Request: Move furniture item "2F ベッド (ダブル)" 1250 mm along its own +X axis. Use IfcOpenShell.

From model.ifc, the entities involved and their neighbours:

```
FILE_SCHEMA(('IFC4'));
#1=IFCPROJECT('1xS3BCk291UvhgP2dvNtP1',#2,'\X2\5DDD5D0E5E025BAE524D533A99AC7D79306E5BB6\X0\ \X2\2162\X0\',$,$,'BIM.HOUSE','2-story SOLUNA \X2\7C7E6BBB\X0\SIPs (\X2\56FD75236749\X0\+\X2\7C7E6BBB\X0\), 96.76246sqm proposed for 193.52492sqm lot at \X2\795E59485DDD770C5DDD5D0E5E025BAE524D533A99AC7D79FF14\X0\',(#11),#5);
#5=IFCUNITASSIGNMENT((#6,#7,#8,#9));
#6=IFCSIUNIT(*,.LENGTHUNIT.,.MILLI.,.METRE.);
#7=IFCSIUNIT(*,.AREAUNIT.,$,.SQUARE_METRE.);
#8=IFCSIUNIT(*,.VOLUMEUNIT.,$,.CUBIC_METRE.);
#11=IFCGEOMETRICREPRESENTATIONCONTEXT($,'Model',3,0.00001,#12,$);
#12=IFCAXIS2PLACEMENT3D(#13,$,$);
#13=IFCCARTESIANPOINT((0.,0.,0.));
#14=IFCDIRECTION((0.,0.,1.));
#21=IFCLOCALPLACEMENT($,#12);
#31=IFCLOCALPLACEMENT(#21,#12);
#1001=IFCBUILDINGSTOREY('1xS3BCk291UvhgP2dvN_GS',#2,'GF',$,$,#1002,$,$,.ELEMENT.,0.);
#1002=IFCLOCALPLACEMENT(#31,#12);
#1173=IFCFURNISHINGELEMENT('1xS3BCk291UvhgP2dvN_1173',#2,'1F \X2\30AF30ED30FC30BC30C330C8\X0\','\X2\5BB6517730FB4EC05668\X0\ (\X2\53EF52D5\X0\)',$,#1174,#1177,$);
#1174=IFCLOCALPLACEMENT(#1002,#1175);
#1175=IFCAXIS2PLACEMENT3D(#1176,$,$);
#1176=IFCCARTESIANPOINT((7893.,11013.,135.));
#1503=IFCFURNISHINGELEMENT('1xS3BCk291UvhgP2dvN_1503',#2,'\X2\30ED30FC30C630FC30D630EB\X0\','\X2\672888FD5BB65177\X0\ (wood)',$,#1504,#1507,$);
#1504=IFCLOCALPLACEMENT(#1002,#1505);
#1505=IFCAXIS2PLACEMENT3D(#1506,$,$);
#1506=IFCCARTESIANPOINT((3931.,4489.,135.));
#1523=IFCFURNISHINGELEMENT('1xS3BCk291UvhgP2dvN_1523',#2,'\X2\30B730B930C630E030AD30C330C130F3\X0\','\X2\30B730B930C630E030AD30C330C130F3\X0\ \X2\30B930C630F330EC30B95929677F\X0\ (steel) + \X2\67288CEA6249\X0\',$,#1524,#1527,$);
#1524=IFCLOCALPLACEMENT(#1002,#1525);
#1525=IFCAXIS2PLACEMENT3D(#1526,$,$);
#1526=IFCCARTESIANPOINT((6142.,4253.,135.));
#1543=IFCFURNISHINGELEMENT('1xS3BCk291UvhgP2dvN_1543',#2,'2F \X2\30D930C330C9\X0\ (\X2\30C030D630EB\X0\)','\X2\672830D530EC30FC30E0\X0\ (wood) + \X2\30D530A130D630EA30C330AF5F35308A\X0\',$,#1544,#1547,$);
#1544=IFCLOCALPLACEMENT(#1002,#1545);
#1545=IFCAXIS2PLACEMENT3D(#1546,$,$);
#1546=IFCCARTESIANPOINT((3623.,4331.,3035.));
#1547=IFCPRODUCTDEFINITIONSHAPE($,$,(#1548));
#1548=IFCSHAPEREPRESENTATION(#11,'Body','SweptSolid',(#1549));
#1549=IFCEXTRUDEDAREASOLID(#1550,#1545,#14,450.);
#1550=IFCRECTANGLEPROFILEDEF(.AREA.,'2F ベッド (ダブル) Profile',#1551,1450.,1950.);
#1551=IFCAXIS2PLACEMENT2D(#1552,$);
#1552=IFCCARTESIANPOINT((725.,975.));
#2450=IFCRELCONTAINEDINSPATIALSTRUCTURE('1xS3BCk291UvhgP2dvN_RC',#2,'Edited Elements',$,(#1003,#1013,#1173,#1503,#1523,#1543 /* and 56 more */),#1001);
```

```python
import ifcopenshell
import ifcopenshell.api.geometry
import ifcopenshell.util.placement

model = ifcopenshell.open("model.ifc")

item = model.by_guid("1xS3BCk291UvhgP2dvN_1543")
matrix = ifcopenshell.util.placement.get_local_placement(item.ObjectPlacement)
matrix[:3, 3] += matrix[:3, 0] * 1250.0
ifcopenshell.api.geometry.edit_object_placement(model, product=item, matrix=matrix, is_si=False)

print(ifcopenshell.util.placement.get_local_placement(item.ObjectPlacement).round(3) + 0.0)

model.write("model_edited.ifc")
```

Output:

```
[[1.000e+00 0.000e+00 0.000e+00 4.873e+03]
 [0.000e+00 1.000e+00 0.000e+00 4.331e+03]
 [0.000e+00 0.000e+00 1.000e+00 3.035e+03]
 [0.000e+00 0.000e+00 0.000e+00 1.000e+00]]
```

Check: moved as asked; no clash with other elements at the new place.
